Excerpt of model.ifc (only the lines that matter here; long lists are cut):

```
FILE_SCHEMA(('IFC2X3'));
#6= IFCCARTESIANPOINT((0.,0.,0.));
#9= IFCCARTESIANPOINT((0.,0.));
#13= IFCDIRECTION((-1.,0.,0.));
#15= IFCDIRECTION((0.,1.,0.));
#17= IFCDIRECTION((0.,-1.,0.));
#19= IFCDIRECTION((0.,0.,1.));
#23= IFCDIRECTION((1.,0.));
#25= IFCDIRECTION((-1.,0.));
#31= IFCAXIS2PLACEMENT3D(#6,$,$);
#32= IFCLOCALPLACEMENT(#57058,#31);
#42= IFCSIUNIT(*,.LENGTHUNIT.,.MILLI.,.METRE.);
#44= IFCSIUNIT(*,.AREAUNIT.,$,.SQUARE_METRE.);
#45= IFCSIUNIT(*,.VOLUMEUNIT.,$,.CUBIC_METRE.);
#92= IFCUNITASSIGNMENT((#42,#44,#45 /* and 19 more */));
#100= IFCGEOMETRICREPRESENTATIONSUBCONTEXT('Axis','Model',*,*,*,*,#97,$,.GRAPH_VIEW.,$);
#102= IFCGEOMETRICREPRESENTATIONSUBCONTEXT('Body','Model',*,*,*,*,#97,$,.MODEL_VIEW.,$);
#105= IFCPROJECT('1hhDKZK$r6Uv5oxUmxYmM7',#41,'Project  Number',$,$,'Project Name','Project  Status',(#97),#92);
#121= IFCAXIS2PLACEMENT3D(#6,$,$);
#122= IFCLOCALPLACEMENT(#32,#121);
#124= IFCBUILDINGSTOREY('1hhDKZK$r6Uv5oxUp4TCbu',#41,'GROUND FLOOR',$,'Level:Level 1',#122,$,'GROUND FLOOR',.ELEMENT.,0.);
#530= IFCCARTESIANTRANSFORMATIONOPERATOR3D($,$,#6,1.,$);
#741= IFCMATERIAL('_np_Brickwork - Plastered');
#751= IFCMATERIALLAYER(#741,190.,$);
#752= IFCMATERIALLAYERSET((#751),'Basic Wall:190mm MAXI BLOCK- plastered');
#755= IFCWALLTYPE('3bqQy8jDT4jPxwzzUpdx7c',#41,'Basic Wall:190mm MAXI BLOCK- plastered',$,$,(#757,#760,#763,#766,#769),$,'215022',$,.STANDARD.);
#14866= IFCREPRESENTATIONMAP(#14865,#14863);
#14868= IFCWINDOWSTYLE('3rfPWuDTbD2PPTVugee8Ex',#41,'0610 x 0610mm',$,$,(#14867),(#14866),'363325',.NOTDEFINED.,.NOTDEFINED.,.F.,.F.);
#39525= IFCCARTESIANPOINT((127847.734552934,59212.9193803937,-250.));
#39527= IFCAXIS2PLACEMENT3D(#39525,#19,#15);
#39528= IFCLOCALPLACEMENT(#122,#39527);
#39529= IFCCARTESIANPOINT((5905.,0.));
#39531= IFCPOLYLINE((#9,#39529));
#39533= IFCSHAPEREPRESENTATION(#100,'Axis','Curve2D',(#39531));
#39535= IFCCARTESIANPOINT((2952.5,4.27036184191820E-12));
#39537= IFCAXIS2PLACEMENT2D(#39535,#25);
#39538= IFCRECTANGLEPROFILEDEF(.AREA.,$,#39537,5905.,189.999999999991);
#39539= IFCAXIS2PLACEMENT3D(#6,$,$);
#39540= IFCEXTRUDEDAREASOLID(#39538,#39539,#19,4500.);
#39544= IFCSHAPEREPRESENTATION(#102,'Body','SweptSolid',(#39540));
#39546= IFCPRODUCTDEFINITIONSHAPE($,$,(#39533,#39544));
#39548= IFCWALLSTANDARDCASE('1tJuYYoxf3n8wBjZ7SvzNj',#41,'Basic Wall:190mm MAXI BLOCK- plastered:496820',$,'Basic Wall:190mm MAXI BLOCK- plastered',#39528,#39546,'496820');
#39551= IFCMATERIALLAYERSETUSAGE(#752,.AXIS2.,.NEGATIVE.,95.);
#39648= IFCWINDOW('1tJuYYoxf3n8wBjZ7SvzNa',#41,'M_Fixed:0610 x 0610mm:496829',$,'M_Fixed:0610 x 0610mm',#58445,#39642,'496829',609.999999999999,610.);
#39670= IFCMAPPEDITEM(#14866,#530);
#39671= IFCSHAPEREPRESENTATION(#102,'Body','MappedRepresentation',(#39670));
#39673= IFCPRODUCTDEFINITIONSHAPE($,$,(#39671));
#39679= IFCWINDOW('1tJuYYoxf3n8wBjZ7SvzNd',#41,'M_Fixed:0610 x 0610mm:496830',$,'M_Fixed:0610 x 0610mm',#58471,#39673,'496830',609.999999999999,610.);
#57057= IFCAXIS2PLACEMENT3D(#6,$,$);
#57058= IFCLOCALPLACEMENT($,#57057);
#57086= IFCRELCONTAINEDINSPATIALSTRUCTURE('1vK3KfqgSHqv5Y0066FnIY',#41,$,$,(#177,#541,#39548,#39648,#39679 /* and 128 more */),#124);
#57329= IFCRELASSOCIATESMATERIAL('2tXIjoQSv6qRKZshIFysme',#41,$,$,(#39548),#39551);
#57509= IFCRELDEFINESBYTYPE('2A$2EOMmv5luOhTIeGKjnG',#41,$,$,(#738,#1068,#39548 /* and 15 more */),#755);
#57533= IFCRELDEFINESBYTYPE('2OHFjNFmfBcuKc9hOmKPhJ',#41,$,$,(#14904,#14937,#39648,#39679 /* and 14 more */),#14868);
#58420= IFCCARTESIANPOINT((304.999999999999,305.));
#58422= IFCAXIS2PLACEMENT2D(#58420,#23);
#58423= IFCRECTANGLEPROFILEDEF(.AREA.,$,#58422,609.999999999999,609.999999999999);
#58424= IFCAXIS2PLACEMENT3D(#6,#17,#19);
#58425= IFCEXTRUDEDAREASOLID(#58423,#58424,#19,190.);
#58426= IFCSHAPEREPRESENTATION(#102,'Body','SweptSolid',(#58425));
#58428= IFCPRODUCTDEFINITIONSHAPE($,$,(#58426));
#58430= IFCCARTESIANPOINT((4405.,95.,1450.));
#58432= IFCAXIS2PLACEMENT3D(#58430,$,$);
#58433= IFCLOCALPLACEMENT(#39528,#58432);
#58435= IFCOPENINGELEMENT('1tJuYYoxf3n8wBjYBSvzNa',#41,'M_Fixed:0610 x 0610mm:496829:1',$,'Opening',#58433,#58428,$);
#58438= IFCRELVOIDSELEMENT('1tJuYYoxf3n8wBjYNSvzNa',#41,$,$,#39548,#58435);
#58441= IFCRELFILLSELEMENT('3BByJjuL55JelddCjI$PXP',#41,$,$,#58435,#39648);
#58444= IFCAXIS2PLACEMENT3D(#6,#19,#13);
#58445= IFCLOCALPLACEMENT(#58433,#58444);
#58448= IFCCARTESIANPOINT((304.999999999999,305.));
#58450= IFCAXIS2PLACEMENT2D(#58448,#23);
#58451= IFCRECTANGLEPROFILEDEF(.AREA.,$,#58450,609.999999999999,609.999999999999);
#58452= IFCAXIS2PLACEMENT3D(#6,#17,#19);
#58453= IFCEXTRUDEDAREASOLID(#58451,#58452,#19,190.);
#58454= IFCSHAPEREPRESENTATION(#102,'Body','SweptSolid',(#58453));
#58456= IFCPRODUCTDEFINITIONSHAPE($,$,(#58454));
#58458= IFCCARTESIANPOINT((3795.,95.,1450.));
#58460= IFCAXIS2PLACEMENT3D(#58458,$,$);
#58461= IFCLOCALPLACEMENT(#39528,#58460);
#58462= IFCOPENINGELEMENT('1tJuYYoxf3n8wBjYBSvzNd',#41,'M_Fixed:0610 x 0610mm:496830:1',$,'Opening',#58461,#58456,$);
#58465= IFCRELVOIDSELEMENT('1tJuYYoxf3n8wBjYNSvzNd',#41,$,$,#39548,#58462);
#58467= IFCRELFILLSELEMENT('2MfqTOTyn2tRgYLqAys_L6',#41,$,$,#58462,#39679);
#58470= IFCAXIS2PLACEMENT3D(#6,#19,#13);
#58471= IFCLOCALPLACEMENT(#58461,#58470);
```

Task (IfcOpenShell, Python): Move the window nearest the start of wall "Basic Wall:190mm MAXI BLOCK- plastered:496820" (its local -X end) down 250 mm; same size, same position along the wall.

```python
import numpy as np
import ifcopenshell
import ifcopenshell.api.geometry
import ifcopenshell.util.placement
import ifcopenshell.util.unit

model = ifcopenshell.open("model.ifc")
unit_scale = ifcopenshell.util.unit.calculate_unit_scale(model)

window = model.by_id(39679)
opening = window.FillsVoids[0].RelatingOpeningElement
dz = -0.25 / unit_scale

shift = np.array([0.0, 0.0, dz])
# The window is placed relative to its opening, so it follows when the opening moves.
matrix = ifcopenshell.util.placement.get_local_placement(opening.ObjectPlacement)
matrix[:3, 3] += shift
ifcopenshell.api.geometry.edit_object_placement(
    model, product=opening, matrix=matrix, is_si=False, should_transform_children=True
)

print(f"moved by {dz * unit_scale:+.3f} m")

model.write("model_updated.ifc")
```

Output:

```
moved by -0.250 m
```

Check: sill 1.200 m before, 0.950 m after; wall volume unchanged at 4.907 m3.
